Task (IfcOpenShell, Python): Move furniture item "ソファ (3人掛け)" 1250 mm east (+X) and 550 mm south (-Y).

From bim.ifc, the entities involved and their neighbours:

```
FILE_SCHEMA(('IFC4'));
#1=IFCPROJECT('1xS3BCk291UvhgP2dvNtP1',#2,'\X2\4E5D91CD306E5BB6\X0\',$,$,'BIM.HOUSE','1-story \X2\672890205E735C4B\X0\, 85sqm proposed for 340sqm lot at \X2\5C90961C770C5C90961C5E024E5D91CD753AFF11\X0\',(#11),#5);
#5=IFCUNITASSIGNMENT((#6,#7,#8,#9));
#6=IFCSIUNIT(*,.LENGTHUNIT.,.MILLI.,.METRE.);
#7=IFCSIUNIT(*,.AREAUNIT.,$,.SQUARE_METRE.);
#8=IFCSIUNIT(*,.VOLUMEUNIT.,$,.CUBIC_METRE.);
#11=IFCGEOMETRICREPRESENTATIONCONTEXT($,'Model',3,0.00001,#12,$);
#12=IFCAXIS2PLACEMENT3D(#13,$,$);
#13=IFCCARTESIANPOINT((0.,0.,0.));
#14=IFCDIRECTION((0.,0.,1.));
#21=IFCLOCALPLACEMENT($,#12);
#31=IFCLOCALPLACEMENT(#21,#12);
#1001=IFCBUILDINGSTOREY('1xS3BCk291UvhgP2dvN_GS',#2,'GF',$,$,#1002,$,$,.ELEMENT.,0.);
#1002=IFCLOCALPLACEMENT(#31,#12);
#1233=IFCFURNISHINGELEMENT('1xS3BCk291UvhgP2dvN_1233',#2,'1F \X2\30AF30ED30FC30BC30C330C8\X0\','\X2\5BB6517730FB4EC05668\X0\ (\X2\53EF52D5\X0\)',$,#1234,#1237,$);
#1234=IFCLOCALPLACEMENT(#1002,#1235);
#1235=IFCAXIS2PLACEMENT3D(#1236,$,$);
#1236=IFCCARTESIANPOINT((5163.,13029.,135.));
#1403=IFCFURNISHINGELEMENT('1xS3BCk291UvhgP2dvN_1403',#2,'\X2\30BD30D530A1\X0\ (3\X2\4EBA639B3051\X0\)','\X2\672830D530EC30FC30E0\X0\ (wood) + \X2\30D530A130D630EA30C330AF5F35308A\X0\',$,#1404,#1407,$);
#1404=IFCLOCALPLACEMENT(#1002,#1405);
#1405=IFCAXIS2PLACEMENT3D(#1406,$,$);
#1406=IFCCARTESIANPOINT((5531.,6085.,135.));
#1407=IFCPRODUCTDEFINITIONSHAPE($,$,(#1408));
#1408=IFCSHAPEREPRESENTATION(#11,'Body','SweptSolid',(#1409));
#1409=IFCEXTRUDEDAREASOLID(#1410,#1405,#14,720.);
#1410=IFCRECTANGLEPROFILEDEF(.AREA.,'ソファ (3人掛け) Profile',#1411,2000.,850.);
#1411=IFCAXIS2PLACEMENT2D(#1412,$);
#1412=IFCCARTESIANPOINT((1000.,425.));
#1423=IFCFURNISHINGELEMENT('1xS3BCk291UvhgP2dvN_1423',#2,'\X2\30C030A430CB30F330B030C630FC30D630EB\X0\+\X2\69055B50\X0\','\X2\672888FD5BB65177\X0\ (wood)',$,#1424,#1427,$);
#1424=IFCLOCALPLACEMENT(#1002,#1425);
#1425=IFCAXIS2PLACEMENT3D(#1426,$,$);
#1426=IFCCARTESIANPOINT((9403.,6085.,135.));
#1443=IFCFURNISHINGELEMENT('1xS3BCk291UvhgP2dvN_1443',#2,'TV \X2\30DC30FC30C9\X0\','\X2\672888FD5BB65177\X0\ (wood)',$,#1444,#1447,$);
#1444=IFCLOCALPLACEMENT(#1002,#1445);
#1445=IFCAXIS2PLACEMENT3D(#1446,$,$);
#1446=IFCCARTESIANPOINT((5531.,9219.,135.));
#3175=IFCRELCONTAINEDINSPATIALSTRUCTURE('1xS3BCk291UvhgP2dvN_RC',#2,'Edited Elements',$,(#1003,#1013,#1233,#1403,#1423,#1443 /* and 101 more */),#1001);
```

```python
import ifcopenshell
import ifcopenshell.api.geometry
import ifcopenshell.util.placement

model = ifcopenshell.open("bim.ifc")

item = model.by_guid("1xS3BCk291UvhgP2dvN_1403")
matrix = ifcopenshell.util.placement.get_local_placement(item.ObjectPlacement)
matrix[0, 3] += 1250.0
matrix[1, 3] -= 550.0
ifcopenshell.api.geometry.edit_object_placement(model, product=item, matrix=matrix, is_si=False)

print(ifcopenshell.util.placement.get_local_placement(item.ObjectPlacement).round(3) + 0.0)

model.write("bim-out.ifc")
```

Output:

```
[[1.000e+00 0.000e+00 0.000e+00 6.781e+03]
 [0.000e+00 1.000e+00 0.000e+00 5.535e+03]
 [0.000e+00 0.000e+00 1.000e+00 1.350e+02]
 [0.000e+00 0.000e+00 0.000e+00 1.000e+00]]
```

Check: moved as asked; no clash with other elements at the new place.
